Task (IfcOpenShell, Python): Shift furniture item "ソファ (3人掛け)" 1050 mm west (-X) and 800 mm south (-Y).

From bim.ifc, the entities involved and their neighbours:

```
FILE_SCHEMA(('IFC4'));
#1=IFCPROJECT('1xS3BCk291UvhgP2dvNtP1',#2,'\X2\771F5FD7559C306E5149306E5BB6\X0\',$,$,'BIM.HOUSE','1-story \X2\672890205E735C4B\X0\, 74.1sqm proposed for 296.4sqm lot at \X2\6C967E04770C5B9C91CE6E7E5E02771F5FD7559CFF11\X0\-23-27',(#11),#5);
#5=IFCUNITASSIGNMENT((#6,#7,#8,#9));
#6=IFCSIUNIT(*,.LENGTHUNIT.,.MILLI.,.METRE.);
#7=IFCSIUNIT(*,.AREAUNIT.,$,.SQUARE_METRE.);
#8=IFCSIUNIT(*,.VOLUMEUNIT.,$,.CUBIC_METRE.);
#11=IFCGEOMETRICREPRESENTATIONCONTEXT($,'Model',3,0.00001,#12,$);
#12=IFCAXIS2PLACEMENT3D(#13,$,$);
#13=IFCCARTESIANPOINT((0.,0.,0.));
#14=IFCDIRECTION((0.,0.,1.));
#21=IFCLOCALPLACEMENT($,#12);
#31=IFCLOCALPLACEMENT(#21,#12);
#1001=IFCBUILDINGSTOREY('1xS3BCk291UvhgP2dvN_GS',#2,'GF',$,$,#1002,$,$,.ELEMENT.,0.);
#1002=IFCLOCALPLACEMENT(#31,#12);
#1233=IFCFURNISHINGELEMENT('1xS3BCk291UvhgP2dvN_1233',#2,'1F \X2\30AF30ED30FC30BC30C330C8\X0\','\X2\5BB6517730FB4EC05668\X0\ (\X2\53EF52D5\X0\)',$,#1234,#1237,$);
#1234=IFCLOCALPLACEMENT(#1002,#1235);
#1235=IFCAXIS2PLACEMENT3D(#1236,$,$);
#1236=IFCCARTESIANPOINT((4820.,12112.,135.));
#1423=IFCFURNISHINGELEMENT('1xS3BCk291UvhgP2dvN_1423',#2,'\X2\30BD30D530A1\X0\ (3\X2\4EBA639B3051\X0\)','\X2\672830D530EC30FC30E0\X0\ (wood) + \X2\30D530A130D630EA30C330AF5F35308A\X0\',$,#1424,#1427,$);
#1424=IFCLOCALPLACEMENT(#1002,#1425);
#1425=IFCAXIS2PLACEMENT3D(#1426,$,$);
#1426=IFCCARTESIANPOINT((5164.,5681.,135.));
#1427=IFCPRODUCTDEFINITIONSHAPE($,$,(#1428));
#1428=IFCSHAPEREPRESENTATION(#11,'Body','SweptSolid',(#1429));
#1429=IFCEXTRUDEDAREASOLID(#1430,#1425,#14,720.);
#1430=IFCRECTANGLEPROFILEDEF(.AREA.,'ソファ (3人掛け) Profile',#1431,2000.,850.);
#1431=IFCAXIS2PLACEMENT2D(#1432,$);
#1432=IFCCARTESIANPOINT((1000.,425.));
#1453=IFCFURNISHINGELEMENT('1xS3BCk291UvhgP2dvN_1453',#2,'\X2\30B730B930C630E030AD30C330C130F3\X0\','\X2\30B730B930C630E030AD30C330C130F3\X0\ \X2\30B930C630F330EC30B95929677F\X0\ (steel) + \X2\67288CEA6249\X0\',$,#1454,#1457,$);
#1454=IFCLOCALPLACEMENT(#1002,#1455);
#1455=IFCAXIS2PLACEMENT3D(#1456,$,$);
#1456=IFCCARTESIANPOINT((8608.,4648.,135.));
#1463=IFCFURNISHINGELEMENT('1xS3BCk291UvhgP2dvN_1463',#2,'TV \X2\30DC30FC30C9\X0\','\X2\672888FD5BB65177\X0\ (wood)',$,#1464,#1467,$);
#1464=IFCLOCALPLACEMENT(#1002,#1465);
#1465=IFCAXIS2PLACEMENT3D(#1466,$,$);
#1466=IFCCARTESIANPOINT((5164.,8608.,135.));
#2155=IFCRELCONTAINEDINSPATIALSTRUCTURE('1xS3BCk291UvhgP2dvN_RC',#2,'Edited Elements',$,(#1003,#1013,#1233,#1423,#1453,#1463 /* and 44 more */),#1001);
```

```python
import ifcopenshell
import ifcopenshell.api.geometry
import ifcopenshell.util.placement
import ifcopenshell.util.unit

model = ifcopenshell.open("bim.ifc")
unit_scale = ifcopenshell.util.unit.calculate_unit_scale(model)

item = model.by_guid("1xS3BCk291UvhgP2dvN_1423")
matrix = ifcopenshell.util.placement.get_local_placement(item.ObjectPlacement)
matrix[0, 3] -= 1.05 / unit_scale
matrix[1, 3] -= 0.8 / unit_scale
ifcopenshell.api.geometry.edit_object_placement(model, product=item, matrix=matrix, is_si=False)

print(ifcopenshell.util.placement.get_local_placement(item.ObjectPlacement).round(3) + 0.0)

model.write("bim_edited.ifc")
```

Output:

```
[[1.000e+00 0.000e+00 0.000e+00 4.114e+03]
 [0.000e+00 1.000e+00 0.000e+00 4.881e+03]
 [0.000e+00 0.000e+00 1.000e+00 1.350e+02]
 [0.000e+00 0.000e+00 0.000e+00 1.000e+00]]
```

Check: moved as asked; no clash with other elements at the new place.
